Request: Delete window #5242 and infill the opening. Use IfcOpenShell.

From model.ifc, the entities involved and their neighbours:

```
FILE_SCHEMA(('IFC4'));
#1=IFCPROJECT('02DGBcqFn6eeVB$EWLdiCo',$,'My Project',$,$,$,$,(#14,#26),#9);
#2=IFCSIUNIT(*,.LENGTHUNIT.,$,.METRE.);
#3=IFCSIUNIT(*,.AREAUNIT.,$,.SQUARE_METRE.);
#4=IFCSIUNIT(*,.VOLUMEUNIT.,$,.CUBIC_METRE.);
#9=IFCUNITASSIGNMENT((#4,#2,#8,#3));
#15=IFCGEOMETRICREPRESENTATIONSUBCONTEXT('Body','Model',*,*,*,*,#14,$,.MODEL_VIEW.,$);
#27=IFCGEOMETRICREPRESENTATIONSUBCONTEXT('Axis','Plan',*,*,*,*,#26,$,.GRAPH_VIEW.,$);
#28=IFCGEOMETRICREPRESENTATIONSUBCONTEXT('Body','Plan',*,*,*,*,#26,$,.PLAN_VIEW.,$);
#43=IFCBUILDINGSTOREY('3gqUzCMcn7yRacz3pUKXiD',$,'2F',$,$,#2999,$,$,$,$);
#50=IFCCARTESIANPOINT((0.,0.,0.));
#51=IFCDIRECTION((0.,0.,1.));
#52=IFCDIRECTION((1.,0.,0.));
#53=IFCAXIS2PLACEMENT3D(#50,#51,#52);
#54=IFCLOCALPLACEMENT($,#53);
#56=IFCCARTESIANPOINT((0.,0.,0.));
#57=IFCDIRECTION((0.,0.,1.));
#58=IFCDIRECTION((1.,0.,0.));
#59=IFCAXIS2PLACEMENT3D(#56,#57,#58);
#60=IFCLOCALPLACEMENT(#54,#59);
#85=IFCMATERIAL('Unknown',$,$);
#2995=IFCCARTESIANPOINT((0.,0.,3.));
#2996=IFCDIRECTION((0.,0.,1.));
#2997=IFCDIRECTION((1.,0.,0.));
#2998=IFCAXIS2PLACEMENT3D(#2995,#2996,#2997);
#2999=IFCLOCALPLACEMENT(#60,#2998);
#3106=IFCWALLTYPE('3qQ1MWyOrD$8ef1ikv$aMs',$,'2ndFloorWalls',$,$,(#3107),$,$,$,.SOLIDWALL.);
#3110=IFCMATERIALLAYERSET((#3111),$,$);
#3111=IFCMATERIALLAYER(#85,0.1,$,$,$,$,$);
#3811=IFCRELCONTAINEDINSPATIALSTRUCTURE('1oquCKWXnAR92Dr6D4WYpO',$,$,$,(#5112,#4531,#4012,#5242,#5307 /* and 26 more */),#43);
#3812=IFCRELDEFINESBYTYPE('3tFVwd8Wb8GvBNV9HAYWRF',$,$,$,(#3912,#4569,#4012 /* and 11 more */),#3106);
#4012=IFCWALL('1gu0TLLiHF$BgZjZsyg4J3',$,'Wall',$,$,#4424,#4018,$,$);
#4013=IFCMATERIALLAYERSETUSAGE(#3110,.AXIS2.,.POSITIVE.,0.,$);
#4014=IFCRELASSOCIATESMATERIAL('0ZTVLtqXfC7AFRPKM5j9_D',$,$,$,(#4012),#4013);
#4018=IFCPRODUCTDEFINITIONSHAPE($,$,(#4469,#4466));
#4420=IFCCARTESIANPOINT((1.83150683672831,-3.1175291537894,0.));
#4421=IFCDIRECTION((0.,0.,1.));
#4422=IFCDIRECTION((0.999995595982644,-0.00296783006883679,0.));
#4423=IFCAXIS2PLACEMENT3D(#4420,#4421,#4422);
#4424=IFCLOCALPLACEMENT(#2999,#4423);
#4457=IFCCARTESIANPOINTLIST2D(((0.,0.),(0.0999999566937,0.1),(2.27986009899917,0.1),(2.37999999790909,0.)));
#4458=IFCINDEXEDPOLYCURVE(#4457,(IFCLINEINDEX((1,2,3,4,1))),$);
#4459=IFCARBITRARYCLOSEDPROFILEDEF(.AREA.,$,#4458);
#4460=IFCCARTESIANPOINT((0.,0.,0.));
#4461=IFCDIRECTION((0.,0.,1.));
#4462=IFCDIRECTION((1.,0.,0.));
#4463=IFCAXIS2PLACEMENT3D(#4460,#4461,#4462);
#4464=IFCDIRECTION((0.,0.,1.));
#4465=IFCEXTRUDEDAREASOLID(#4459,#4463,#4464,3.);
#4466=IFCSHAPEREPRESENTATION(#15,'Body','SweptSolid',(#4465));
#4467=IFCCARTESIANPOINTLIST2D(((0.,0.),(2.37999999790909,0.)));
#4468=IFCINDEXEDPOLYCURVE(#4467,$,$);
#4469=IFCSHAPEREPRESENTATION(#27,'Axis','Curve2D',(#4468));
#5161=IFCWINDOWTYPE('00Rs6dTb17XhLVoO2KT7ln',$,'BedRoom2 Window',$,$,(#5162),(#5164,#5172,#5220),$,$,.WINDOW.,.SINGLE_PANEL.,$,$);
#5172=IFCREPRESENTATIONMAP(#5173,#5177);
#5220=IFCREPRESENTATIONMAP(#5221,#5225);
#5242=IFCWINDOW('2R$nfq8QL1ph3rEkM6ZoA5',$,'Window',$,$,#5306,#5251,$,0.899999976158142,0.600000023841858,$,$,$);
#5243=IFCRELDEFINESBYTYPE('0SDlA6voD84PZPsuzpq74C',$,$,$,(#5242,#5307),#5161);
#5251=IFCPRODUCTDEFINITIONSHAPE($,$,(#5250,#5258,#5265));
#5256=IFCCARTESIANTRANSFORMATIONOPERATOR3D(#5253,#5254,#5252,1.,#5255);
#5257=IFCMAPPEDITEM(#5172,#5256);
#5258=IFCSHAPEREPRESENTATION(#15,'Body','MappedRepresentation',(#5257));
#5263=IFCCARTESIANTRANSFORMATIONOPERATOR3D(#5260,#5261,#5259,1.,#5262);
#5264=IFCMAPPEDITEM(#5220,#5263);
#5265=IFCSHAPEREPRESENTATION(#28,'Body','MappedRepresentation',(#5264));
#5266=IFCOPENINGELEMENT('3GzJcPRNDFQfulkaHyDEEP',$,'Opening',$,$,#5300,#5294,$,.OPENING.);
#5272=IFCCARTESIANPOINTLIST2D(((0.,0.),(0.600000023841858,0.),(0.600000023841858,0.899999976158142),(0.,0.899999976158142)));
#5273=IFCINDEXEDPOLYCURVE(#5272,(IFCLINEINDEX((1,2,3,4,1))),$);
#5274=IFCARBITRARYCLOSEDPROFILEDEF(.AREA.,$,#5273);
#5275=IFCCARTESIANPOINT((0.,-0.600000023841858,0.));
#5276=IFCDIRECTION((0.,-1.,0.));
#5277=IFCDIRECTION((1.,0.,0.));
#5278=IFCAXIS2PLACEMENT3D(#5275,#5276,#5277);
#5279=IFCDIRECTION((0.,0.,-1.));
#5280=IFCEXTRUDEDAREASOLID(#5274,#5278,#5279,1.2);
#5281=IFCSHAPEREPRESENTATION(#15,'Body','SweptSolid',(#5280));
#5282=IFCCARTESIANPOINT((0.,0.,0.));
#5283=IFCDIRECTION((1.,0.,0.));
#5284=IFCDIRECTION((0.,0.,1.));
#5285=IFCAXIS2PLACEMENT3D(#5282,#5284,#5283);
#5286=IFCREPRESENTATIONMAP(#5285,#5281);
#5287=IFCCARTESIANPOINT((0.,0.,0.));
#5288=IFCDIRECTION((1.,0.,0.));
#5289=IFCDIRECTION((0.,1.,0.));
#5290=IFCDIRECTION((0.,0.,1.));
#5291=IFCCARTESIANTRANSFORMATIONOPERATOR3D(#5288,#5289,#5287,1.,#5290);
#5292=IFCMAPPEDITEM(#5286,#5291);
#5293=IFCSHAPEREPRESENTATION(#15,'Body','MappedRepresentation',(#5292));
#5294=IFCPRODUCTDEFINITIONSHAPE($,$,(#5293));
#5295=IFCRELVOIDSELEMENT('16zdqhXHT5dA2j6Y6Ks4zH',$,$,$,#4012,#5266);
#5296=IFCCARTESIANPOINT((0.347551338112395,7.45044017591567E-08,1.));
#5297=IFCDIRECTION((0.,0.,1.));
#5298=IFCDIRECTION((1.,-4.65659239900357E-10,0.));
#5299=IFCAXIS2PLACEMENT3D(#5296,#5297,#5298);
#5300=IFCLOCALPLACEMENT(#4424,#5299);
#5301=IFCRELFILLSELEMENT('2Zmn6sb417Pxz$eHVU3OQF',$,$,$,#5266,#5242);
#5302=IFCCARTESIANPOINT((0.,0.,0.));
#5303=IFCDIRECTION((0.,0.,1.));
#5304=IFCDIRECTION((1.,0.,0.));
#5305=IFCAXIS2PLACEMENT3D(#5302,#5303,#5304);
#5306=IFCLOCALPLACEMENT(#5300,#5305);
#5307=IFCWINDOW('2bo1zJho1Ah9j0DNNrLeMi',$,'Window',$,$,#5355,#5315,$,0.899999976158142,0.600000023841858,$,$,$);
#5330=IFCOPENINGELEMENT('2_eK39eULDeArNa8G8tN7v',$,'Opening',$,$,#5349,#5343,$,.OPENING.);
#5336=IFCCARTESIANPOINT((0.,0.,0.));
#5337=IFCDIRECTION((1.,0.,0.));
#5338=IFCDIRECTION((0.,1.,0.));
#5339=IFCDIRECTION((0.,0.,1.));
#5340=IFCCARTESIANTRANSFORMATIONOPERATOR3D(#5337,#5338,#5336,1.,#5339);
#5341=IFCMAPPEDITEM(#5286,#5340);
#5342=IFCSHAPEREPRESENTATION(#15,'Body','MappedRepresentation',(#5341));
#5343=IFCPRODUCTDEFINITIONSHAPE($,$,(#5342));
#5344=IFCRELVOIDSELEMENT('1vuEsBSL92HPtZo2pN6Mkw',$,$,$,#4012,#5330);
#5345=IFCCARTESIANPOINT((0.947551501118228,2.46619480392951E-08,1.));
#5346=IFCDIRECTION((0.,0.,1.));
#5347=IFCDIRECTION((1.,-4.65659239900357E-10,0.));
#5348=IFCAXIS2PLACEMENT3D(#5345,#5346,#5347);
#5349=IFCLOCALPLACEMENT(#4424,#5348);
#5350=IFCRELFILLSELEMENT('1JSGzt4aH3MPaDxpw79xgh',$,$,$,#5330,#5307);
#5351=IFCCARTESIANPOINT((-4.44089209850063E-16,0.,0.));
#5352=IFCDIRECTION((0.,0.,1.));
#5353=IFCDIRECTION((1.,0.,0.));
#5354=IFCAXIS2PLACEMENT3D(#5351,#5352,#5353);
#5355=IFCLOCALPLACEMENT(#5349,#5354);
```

```python
import ifcopenshell
import ifcopenshell.api.feature
import ifcopenshell.api.root
import ifcopenshell.geom
import ifcopenshell.util.shape

model = ifcopenshell.open("model.ifc")
settings = ifcopenshell.geom.settings()


def volume(element):
    """Net volume in cubic metres, openings subtracted."""
    shape = ifcopenshell.geom.create_shape(settings, element)
    return ifcopenshell.util.shape.get_volume(shape.geometry)


window = model.by_guid("2R$nfq8QL1ph3rEkM6ZoA5")
opening = window.FillsVoids[0].RelatingOpeningElement
wall = opening.VoidsElements[0].RelatingBuildingElement
before = volume(wall)

ifcopenshell.api.root.remove_product(model, product=window)
ifcopenshell.api.feature.remove_feature(model, feature=opening)

after = volume(wall)

print(f"wall volume {before:.3f} -> {after:.3f} m3")

model.write("model_v2.ifc")
```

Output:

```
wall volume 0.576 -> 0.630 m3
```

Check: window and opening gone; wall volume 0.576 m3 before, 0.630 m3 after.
